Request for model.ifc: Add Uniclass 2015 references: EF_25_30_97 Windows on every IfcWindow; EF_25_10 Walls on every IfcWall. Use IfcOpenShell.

First a look at what the model holds.

```python
import ifcopenshell

model = ifcopenshell.open("model.ifc")
print(model.schema)
print("classifications:", [c.Name for c in model.by_type("IfcClassification")])
for ifc_class in ("IfcDoor", "IfcRoof", "IfcStair", "IfcWall", "IfcWindow"):
    print(ifc_class, len(model.by_type(ifc_class)))
```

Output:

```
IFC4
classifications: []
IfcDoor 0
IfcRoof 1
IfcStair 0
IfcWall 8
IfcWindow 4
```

```python
import ifcopenshell
import ifcopenshell.api.classification

model = ifcopenshell.open("model.ifc")

system = ifcopenshell.api.classification.add_classification(model, classification="Uniclass 2015")

codes = {
    "IfcWindow": ("EF_25_30_97", "Windows"),
    "IfcWall": ("EF_25_10", "Walls"),
}
for ifc_class, (code, name) in codes.items():
    products = model.by_type(ifc_class)
    ifcopenshell.api.classification.add_reference(
        model, products=products, classification=system, identification=code, name=name
    )
    print(code, len(products))

model.write("model_updated.ifc")
```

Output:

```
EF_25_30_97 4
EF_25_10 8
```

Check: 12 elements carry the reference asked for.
